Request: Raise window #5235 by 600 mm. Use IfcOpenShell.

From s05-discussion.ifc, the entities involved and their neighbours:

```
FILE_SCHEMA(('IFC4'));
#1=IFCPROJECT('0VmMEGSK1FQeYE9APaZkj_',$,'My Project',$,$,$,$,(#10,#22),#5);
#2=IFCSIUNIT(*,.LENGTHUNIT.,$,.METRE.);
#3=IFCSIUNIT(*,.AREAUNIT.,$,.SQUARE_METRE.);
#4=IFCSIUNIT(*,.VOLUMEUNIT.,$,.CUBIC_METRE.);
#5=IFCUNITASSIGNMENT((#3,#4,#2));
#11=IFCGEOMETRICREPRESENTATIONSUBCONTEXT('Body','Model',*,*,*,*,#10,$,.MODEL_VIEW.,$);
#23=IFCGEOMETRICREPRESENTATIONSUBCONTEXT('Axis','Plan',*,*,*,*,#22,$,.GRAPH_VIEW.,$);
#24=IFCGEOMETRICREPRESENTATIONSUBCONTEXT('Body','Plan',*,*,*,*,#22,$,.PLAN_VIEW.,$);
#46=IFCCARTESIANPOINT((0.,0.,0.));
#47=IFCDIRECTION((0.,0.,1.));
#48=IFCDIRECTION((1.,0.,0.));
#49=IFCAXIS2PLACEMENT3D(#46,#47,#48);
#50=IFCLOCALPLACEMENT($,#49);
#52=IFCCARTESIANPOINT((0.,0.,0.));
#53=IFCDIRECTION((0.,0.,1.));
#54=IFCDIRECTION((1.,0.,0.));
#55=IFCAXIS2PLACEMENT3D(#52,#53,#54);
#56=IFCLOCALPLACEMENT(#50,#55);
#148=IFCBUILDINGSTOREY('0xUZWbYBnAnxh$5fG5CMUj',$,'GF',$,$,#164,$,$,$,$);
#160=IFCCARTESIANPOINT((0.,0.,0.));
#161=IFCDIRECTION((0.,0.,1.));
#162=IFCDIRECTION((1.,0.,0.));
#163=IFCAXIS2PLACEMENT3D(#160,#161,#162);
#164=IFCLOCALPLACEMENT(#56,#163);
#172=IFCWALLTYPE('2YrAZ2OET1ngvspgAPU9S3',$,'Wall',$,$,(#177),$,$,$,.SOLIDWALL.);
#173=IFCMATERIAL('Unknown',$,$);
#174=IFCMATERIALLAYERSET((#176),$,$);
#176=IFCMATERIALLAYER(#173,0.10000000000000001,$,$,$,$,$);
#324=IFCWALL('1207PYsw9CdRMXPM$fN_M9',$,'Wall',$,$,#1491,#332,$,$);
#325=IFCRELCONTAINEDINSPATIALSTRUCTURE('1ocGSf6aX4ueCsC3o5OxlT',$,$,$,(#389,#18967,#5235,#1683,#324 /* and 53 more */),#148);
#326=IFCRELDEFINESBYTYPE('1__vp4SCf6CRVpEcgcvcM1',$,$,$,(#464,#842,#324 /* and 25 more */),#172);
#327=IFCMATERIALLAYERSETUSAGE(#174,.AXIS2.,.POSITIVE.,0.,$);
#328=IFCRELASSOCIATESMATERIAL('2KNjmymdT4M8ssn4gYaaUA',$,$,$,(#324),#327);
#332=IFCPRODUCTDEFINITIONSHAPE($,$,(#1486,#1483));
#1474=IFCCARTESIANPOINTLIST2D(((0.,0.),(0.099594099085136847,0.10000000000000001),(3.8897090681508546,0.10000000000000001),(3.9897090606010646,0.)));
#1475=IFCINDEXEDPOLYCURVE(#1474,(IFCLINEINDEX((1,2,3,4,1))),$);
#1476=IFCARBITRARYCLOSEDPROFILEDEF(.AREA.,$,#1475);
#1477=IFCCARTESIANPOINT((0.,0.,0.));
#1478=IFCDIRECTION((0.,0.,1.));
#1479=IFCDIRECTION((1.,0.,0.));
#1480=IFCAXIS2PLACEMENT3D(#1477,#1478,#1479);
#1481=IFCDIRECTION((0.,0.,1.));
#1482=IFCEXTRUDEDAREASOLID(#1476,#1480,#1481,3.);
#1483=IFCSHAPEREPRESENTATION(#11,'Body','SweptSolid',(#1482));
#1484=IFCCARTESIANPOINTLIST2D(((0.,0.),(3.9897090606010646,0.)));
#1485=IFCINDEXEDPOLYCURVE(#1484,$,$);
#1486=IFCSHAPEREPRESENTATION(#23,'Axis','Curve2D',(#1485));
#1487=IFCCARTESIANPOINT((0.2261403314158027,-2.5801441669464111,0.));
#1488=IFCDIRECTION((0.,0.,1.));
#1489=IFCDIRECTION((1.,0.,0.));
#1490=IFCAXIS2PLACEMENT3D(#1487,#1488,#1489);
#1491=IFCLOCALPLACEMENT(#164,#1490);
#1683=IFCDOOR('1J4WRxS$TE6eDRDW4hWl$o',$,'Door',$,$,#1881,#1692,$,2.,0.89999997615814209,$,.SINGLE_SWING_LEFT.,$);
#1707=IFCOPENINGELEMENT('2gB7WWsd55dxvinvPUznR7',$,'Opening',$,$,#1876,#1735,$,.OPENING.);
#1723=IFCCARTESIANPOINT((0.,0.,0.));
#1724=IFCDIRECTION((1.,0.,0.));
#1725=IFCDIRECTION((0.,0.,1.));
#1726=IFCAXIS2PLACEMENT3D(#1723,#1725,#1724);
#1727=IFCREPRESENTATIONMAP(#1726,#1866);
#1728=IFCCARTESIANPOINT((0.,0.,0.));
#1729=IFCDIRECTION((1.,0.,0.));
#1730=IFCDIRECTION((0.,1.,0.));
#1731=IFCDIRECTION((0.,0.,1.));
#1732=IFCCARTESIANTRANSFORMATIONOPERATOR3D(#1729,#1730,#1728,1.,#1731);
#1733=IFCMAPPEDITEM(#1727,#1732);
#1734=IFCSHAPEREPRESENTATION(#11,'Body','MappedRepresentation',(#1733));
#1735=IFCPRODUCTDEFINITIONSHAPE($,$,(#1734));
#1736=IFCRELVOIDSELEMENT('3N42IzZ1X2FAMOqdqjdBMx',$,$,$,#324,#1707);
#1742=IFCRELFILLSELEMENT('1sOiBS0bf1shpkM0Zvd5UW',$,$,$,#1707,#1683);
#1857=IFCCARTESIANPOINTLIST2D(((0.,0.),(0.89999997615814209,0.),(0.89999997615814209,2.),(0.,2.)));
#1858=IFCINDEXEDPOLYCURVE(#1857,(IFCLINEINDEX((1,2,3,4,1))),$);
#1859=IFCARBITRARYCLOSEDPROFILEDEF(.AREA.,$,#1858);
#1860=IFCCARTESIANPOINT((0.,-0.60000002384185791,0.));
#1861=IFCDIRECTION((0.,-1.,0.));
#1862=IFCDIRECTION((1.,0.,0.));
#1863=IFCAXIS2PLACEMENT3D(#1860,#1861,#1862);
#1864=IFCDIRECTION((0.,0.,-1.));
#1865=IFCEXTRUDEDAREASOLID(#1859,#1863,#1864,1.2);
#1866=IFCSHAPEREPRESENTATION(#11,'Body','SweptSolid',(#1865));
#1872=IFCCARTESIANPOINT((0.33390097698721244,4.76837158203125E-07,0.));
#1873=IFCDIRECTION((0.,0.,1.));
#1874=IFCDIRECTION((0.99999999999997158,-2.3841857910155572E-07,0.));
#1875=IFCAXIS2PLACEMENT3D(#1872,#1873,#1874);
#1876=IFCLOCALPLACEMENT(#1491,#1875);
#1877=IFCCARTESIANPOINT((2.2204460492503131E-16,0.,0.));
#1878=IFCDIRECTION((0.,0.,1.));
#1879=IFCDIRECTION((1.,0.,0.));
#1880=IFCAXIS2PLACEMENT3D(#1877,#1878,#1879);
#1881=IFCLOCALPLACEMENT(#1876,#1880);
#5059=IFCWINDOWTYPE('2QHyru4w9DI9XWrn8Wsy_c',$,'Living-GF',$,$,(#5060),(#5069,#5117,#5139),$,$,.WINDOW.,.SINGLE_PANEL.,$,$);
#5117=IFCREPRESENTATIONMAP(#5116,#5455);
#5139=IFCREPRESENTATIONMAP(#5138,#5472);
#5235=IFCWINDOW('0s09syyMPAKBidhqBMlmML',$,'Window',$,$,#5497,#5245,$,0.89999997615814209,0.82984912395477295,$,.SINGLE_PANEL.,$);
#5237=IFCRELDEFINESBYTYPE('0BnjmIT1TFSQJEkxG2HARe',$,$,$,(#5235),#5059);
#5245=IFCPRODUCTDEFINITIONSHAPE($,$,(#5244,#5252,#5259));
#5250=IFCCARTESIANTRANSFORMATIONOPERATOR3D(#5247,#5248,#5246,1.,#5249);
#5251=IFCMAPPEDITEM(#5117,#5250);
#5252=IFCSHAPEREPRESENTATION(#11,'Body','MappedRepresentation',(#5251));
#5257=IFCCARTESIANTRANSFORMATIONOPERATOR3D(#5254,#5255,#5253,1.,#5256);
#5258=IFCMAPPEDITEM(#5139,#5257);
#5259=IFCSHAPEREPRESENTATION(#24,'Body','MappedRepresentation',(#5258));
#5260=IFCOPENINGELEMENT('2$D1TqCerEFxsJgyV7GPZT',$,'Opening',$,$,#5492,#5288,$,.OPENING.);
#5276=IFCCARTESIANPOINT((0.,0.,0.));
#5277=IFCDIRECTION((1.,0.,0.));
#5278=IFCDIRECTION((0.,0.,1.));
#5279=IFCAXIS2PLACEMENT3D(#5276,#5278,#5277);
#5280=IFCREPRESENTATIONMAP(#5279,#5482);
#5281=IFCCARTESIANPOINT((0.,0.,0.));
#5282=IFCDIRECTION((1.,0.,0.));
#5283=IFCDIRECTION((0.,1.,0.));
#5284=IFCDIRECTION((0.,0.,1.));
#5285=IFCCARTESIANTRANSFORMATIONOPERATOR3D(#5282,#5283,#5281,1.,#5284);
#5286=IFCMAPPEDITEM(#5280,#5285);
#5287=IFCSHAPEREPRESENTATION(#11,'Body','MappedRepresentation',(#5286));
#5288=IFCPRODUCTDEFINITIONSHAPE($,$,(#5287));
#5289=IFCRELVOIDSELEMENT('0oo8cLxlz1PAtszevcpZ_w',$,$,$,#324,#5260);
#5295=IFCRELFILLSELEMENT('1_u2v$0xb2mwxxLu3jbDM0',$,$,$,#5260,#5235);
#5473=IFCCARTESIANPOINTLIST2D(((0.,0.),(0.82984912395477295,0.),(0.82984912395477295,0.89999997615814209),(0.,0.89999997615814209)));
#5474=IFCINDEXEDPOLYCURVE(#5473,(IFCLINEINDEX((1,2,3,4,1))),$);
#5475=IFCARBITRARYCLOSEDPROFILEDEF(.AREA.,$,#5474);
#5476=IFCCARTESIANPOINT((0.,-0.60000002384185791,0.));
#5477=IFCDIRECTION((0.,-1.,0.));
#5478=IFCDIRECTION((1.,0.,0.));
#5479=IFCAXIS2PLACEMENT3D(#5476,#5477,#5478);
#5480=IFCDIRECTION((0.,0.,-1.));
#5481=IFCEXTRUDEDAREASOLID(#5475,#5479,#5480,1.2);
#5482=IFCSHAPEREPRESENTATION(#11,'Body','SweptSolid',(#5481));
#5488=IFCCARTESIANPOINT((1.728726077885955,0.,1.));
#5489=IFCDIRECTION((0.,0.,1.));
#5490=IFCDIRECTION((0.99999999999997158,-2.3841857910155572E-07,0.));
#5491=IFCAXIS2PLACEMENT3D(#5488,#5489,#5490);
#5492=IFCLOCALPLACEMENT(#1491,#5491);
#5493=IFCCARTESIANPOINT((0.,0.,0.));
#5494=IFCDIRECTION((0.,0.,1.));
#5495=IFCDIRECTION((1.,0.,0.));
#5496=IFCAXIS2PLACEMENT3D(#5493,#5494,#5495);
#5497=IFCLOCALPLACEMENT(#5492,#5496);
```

```python
import numpy as np
import ifcopenshell
import ifcopenshell.api.geometry
import ifcopenshell.util.placement
import ifcopenshell.util.unit

model = ifcopenshell.open("s05-discussion.ifc")
unit_scale = ifcopenshell.util.unit.calculate_unit_scale(model)

window = model.by_guid("0s09syyMPAKBidhqBMlmML")
opening = window.FillsVoids[0].RelatingOpeningElement
dz = 0.6 / unit_scale

shift = np.array([0.0, 0.0, dz])
# The window is placed relative to its opening, so it follows when the opening moves.
matrix = ifcopenshell.util.placement.get_local_placement(opening.ObjectPlacement)
matrix[:3, 3] += shift
ifcopenshell.api.geometry.edit_object_placement(
    model, product=opening, matrix=matrix, is_si=False, should_transform_children=True
)

print(f"moved by {dz * unit_scale:+.3f} m")

model.write("s05-discussion_v2.ifc")
```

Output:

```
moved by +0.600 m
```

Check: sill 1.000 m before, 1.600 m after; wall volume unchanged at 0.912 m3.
